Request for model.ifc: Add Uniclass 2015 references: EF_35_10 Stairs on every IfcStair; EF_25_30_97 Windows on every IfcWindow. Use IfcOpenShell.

First a look at what the model holds.

```python
import ifcopenshell

model = ifcopenshell.open("model.ifc")
print(model.schema)
print("classifications:", [c.Name for c in model.by_type("IfcClassification")])
for ifc_class in ("IfcDoor", "IfcRoof", "IfcStair", "IfcWall", "IfcWindow"):
    print(ifc_class, len(model.by_type(ifc_class)))
```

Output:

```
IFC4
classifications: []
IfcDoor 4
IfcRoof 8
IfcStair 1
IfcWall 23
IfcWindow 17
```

```python
import ifcopenshell
import ifcopenshell.api.classification

model = ifcopenshell.open("model.ifc")

system = ifcopenshell.api.classification.add_classification(model, classification="Uniclass 2015")

codes = {
    "IfcStair": ("EF_35_10", "Stairs"),
    "IfcWindow": ("EF_25_30_97", "Windows"),
}
for ifc_class, (code, name) in codes.items():
    products = model.by_type(ifc_class)
    ifcopenshell.api.classification.add_reference(
        model, products=products, classification=system, identification=code, name=name
    )
    print(code, len(products))

model.write("model_rev.ifc")
```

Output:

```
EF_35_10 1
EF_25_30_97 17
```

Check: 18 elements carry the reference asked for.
